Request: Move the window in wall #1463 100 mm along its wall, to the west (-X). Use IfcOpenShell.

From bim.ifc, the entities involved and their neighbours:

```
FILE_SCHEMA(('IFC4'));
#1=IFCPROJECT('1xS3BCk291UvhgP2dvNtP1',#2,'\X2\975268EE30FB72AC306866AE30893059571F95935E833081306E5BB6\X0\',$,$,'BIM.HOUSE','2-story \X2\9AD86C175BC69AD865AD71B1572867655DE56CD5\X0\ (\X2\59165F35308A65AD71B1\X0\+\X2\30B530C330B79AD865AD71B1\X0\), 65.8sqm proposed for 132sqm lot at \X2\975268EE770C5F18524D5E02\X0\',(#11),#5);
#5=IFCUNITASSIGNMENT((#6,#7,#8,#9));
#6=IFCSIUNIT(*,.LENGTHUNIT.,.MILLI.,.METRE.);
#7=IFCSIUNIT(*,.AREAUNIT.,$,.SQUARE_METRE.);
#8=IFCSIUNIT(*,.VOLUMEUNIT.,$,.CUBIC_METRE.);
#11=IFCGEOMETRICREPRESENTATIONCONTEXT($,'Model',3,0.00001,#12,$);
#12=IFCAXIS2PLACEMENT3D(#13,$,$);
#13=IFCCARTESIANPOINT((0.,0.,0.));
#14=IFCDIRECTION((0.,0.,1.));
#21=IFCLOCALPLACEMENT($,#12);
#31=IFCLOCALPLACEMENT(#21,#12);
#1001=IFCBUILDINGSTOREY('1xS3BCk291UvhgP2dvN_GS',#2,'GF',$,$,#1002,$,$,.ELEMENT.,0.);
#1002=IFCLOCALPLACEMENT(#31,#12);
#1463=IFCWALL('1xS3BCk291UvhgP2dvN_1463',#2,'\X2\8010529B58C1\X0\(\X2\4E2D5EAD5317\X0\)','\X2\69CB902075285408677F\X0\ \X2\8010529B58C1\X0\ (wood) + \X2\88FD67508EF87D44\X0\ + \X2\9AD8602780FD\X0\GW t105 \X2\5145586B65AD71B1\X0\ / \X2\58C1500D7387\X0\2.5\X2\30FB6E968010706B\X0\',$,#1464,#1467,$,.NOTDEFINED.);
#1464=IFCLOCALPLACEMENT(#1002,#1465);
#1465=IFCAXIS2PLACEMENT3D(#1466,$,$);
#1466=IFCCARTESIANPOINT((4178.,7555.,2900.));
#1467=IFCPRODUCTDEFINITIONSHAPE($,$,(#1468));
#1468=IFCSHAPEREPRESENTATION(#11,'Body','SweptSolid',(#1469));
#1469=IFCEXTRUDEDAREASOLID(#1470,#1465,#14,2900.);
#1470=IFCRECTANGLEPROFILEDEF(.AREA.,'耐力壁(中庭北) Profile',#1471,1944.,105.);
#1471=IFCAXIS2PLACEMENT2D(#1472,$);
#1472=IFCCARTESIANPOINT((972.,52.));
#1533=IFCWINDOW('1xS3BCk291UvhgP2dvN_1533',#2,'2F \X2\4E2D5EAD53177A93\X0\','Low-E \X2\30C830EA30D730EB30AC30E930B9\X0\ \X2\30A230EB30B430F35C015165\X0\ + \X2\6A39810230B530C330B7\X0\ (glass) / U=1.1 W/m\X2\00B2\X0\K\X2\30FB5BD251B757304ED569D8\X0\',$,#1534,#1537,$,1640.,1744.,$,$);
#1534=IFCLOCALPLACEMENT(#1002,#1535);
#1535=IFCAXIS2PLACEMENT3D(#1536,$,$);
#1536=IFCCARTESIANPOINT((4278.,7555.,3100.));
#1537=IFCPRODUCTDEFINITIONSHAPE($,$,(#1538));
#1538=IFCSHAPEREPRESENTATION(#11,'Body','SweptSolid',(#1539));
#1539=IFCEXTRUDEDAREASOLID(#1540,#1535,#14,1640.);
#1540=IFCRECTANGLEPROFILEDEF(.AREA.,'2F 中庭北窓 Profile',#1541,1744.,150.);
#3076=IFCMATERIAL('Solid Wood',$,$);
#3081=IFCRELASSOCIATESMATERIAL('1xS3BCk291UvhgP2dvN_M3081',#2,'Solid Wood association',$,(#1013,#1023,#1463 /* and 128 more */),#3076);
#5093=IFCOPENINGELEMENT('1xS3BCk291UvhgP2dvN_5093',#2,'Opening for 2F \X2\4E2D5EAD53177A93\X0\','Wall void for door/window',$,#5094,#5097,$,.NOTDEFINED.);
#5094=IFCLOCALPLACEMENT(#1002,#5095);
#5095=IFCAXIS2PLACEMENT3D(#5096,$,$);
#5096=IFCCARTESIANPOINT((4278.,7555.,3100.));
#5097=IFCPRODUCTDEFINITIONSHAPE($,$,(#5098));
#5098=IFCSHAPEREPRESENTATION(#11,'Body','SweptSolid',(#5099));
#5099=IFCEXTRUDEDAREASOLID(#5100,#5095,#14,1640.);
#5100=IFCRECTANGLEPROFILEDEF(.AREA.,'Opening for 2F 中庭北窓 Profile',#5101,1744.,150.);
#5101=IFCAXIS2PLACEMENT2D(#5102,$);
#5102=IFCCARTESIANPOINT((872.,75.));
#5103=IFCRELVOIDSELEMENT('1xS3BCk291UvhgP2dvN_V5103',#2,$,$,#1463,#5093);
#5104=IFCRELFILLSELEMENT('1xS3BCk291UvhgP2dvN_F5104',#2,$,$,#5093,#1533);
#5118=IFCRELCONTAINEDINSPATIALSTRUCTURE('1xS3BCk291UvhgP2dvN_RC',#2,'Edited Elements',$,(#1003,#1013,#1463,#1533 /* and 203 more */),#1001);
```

```python
import ifcopenshell
import ifcopenshell.api.geometry
import ifcopenshell.util.placement

model = ifcopenshell.open("bim.ifc")

window = model.by_guid("1xS3BCk291UvhgP2dvN_1533")
opening = window.FillsVoids[0].RelatingOpeningElement
wall = opening.VoidsElements[0].RelatingBuildingElement

wall_matrix = ifcopenshell.util.placement.get_local_placement(wall.ObjectPlacement)
shift = wall_matrix[:3, 0] * -100.0
before = ifcopenshell.util.placement.get_local_placement(window.ObjectPlacement)[:3, 3].copy()

# The window is not placed relative to its opening, so move both.
for product in (opening, window):
    matrix = ifcopenshell.util.placement.get_local_placement(product.ObjectPlacement)
    matrix[:3, 3] += shift
    ifcopenshell.api.geometry.edit_object_placement(model, product=product, matrix=matrix, is_si=False)

after = ifcopenshell.util.placement.get_local_placement(window.ObjectPlacement)[:3, 3]
print("window moved by", (after - before).round(3) + 0.0)

model.write("bim_v2.ifc")
```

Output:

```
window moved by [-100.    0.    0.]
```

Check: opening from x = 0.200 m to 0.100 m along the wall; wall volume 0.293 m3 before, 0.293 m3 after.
